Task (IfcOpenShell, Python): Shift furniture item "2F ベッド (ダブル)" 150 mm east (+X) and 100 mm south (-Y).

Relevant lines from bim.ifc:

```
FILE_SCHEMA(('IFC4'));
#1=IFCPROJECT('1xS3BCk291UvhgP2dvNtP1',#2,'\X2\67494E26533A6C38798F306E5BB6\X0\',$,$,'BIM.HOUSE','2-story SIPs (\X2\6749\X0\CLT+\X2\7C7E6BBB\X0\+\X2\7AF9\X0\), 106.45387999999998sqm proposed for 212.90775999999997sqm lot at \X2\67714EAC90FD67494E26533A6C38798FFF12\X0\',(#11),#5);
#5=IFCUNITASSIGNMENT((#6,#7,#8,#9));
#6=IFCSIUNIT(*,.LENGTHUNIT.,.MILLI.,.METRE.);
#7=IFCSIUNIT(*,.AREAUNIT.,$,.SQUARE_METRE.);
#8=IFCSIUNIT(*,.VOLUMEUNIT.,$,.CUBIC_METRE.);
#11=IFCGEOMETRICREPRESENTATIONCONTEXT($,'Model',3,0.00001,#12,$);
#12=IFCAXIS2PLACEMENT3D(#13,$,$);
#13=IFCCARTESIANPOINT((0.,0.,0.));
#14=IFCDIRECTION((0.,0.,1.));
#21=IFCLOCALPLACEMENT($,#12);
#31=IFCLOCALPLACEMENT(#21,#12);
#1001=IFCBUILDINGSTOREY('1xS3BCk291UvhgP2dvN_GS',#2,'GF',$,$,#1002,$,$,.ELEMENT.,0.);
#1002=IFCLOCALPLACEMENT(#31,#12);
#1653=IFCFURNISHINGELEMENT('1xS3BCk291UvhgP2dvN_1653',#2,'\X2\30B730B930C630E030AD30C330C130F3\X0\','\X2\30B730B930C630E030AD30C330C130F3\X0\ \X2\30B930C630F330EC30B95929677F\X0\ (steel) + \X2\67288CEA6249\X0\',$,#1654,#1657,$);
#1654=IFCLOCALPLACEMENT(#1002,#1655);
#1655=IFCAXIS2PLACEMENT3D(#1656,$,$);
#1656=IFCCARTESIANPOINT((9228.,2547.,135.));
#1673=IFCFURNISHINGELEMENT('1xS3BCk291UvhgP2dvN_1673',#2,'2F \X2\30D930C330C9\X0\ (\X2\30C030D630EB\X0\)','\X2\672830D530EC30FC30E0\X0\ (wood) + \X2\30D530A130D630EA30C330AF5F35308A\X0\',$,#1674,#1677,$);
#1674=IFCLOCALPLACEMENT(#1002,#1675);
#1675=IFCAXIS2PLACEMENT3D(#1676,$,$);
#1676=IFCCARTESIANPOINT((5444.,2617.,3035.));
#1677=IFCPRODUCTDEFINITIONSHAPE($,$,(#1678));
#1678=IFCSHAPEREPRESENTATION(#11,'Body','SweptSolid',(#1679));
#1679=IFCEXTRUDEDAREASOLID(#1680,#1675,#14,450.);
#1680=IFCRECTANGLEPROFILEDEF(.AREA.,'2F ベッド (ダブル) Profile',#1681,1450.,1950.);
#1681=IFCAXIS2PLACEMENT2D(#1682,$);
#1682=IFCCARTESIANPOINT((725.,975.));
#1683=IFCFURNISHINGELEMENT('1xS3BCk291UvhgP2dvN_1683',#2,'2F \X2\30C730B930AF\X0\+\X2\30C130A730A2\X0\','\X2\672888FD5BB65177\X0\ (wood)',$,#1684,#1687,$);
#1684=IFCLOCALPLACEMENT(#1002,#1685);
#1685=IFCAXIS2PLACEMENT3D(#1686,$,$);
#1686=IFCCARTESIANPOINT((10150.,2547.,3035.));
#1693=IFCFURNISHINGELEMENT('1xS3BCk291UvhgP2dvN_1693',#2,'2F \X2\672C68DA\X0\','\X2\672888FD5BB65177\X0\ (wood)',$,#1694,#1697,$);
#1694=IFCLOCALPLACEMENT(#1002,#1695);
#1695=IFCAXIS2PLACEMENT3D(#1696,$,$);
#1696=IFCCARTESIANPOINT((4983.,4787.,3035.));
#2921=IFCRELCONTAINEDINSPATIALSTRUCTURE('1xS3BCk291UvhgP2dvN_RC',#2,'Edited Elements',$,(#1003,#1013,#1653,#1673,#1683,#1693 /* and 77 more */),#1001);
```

```python
import ifcopenshell
import ifcopenshell.api.geometry
import ifcopenshell.util.placement
import ifcopenshell.util.unit

model = ifcopenshell.open("bim.ifc")
unit_scale = ifcopenshell.util.unit.calculate_unit_scale(model)

item = model.by_id(1673)
matrix = ifcopenshell.util.placement.get_local_placement(item.ObjectPlacement)
matrix[0, 3] += 0.15 / unit_scale
matrix[1, 3] -= 0.1 / unit_scale
ifcopenshell.api.geometry.edit_object_placement(model, product=item, matrix=matrix, is_si=False)

print(ifcopenshell.util.placement.get_local_placement(item.ObjectPlacement).round(3) + 0.0)

model.write("bim_edited.ifc")
```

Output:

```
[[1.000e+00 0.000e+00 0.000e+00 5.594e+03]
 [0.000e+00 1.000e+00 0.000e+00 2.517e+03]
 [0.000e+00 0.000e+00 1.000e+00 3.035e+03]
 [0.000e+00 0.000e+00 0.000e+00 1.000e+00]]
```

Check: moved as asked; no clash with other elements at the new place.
